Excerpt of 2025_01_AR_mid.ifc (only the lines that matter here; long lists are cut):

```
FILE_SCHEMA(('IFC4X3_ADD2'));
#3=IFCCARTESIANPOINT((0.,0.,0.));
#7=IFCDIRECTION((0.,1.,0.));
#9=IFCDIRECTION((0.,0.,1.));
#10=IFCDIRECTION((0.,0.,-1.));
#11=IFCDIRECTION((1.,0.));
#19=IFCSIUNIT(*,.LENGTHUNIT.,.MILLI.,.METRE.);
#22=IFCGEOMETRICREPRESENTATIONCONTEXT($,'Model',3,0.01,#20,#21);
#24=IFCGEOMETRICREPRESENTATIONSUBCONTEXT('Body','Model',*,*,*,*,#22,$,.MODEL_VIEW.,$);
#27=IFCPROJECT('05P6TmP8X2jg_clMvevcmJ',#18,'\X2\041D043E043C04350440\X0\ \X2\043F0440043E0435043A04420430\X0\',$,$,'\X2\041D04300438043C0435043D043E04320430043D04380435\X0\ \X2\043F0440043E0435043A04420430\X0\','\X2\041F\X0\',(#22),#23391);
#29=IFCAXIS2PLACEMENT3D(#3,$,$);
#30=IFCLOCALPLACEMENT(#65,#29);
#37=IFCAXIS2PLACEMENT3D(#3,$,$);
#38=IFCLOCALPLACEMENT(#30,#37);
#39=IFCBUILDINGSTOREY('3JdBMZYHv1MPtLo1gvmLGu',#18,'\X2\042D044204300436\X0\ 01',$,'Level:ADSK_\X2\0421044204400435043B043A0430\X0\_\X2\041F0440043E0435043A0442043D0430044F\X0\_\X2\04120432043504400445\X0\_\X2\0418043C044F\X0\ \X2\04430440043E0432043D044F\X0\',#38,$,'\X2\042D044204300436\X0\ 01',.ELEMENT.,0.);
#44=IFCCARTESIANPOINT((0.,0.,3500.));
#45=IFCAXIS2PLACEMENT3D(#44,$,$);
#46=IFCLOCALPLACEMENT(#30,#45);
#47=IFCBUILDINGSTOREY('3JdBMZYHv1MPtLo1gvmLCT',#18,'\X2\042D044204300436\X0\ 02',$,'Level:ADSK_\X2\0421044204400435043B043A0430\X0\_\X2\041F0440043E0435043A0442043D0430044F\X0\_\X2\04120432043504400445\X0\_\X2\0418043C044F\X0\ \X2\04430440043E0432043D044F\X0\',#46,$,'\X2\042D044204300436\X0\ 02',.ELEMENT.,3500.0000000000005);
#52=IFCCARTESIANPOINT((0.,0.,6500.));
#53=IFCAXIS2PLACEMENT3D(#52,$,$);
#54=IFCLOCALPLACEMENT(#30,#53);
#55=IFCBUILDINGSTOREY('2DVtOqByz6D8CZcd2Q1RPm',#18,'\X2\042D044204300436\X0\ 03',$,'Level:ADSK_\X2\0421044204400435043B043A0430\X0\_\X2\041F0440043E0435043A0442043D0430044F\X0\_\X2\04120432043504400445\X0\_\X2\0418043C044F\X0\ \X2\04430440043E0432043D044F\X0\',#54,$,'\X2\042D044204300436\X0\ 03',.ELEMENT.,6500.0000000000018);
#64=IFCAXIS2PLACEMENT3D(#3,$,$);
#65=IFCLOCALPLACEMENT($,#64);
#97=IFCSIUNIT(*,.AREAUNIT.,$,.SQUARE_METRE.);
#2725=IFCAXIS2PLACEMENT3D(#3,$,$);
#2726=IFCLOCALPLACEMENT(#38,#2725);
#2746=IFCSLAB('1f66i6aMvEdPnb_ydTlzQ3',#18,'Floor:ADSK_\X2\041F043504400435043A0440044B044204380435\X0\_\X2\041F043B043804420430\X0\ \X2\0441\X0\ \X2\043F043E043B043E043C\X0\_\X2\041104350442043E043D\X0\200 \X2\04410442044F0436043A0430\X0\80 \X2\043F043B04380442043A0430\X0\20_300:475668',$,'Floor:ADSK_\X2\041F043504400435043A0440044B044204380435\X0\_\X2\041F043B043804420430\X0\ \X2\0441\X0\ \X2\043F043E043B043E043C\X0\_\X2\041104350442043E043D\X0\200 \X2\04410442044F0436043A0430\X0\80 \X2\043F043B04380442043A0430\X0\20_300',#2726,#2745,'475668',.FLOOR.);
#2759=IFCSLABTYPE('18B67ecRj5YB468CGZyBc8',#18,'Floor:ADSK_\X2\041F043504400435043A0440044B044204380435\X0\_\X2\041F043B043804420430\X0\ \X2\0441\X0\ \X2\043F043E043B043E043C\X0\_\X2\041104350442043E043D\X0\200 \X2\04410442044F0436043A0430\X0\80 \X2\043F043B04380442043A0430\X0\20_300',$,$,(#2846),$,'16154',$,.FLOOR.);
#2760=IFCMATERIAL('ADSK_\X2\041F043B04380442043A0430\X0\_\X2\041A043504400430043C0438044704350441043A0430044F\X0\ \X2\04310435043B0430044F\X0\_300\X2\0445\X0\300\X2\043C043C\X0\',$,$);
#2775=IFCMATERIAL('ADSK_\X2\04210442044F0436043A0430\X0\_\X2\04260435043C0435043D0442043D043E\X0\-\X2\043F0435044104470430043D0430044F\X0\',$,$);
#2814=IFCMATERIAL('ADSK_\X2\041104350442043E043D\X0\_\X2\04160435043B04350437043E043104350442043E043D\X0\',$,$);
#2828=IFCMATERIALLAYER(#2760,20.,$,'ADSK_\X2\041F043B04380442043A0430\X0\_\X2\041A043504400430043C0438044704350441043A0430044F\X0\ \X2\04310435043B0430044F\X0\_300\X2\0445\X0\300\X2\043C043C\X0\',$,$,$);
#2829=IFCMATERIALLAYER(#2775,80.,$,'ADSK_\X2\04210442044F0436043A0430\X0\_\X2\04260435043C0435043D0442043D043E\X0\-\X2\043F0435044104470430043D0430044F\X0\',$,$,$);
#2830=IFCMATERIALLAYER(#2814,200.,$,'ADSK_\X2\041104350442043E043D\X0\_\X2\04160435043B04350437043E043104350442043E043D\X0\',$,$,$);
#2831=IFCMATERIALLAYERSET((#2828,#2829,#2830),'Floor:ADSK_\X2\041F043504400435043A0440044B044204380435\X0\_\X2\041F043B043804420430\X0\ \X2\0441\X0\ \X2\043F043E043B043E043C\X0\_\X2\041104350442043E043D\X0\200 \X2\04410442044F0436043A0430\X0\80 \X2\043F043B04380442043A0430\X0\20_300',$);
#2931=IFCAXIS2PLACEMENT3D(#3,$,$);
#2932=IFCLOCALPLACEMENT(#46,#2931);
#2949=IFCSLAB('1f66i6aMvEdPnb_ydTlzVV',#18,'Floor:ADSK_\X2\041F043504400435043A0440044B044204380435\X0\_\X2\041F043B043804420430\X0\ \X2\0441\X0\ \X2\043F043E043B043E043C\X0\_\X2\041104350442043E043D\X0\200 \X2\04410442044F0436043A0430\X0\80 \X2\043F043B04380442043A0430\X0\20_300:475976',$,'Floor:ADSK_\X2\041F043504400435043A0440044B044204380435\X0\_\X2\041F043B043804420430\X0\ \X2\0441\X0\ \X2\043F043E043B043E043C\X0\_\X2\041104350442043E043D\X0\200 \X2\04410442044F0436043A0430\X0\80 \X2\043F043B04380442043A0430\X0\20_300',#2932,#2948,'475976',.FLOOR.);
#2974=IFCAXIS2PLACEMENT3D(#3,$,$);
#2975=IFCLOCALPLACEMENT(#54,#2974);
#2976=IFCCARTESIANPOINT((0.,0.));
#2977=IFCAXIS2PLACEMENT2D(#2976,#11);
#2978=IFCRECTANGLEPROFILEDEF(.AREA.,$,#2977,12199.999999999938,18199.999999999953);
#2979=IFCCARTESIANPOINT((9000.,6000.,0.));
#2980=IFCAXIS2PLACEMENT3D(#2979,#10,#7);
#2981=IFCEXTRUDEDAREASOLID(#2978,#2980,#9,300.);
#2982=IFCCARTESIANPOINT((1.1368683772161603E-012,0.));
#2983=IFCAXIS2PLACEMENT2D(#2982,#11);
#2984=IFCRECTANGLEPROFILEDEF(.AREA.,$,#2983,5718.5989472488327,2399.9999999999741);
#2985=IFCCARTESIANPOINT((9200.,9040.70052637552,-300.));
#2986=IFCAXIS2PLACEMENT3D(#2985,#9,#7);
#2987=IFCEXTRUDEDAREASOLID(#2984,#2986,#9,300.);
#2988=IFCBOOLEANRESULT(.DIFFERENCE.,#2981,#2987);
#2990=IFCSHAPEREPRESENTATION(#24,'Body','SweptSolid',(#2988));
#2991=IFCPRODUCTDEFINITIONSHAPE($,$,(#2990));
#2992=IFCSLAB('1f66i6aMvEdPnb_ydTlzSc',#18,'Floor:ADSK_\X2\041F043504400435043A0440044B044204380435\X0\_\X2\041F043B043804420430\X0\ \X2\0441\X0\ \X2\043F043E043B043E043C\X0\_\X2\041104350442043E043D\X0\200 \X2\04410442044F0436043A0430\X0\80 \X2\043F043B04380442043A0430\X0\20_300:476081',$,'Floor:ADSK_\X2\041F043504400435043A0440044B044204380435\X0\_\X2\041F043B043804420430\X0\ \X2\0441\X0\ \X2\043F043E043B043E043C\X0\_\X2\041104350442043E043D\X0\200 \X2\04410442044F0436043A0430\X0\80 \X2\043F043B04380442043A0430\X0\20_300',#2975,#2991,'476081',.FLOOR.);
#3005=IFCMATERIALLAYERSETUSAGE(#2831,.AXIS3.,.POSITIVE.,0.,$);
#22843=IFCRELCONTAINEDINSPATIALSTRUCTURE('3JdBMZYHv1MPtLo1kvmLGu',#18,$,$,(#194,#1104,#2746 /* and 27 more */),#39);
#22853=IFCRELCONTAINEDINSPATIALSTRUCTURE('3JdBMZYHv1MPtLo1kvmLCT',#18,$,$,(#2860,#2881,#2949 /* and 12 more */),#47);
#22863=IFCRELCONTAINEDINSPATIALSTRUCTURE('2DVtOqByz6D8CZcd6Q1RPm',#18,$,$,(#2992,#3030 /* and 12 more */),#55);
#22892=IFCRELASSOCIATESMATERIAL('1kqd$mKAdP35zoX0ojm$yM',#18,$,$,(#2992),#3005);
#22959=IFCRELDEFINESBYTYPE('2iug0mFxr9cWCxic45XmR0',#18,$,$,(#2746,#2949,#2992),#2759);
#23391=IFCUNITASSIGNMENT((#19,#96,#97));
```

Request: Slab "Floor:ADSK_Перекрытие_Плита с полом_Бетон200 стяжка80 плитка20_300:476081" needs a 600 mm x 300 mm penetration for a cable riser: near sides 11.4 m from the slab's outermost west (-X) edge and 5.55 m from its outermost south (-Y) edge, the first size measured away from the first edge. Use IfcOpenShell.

```python
import numpy as np
import ifcopenshell
import ifcopenshell.api.feature
import ifcopenshell.api.geometry
import ifcopenshell.api.root
import ifcopenshell.geom
import ifcopenshell.util.placement
import ifcopenshell.util.representation
import ifcopenshell.util.shape
import ifcopenshell.util.unit

model = ifcopenshell.open("2025_01_AR_mid.ifc")
unit_scale = ifcopenshell.util.unit.calculate_unit_scale(model)
settings = ifcopenshell.geom.settings()


def volume(element):
    """Net volume in cubic metres, openings subtracted."""
    shape = ifcopenshell.geom.create_shape(settings, element)
    return ifcopenshell.util.shape.get_volume(shape.geometry)


slab = model.by_guid("1f66i6aMvEdPnb_ydTlzSc")
before = volume(slab)

# Extent in the slab's own axes, in metres. The edges named are its -X and -Y sides.
slab_shape = ifcopenshell.geom.create_shape(settings, slab)
vertices = ifcopenshell.util.shape.get_vertices(slab_shape.geometry)
x_min, y_min, bottom = vertices.min(axis=0)
top = vertices[:, 2].max()

opening = ifcopenshell.api.root.create_entity(model, ifc_class="IfcOpeningElement", name="Cable riser opening", predefined_type="OPENING")
context = ifcopenshell.util.representation.get_context(model, "Model", "Body", "MODEL_VIEW")
width, depth = 0.6, 0.3
outline = [(0.0, 0.0), (width, 0.0), (width, depth), (0.0, depth), (0.0, 0.0)]
# Overshoot both faces by 50 mm so the cut is clean.
shape = ifcopenshell.api.geometry.add_slab_representation(
    model, context=context, depth=top - bottom + 0.1, polyline=outline
)
ifcopenshell.api.geometry.assign_representation(model, product=opening, representation=shape)

matrix = ifcopenshell.util.placement.get_local_placement(slab.ObjectPlacement)
matrix[:, 3] = matrix @ np.append(np.array([x_min + 11.4, y_min + 5.55, bottom - 0.05]) / unit_scale, 1.0)
ifcopenshell.api.geometry.edit_object_placement(model, product=opening, matrix=matrix, is_si=False)
ifcopenshell.api.feature.add_feature(model, feature=opening, element=slab)

after = volume(slab)

print(f"slab volume {before:.3f} -> {after:.3f} m3")

model.write("2025_01_AR_mid_edited.ifc")
```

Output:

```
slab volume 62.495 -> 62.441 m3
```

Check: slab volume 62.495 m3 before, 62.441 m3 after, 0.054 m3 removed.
